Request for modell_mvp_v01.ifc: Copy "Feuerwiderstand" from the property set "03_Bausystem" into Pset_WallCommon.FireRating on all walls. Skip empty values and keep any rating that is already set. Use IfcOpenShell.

First a look at what the model holds.

```python
import ifcopenshell
import ifcopenshell.util.element

model = ifcopenshell.open("modell_mvp_v01.ifc")
print(model.schema)
walls = model.by_type("IfcWall")
print(len(walls), "walls")
for e in walls[:8]:
    source = ifcopenshell.util.element.get_pset(e, "03_Bausystem", "Feuerwiderstand")
    target = ifcopenshell.util.element.get_pset(e, "Pset_WallCommon", "FireRating")
    print(e.id(), repr(source), repr(target), sep=" | ")
```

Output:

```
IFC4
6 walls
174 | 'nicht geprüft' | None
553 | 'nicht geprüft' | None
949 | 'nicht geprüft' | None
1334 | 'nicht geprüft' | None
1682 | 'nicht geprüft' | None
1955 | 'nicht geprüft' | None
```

```python
import ifcopenshell
import ifcopenshell.api.pset
import ifcopenshell.util.element

model = ifcopenshell.open("modell_mvp_v01.ifc")

count = 0
for e in model.by_type("IfcWall"):
    value = ifcopenshell.util.element.get_pset(e, "03_Bausystem", "Feuerwiderstand")
    current = ifcopenshell.util.element.get_pset(e, "Pset_WallCommon", "FireRating")
    if not value or not value.strip() or current:
        continue
    # add_pset returns the element's existing set when there is one.
    pset = ifcopenshell.api.pset.add_pset(model, product=e, name="Pset_WallCommon")
    ifcopenshell.api.pset.edit_pset(model, pset=pset, properties={"FireRating": value})
    count += 1

print(count, "walls updated")

model.write("modell_mvp_v01_updated.ifc")
```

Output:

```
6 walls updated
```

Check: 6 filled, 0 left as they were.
